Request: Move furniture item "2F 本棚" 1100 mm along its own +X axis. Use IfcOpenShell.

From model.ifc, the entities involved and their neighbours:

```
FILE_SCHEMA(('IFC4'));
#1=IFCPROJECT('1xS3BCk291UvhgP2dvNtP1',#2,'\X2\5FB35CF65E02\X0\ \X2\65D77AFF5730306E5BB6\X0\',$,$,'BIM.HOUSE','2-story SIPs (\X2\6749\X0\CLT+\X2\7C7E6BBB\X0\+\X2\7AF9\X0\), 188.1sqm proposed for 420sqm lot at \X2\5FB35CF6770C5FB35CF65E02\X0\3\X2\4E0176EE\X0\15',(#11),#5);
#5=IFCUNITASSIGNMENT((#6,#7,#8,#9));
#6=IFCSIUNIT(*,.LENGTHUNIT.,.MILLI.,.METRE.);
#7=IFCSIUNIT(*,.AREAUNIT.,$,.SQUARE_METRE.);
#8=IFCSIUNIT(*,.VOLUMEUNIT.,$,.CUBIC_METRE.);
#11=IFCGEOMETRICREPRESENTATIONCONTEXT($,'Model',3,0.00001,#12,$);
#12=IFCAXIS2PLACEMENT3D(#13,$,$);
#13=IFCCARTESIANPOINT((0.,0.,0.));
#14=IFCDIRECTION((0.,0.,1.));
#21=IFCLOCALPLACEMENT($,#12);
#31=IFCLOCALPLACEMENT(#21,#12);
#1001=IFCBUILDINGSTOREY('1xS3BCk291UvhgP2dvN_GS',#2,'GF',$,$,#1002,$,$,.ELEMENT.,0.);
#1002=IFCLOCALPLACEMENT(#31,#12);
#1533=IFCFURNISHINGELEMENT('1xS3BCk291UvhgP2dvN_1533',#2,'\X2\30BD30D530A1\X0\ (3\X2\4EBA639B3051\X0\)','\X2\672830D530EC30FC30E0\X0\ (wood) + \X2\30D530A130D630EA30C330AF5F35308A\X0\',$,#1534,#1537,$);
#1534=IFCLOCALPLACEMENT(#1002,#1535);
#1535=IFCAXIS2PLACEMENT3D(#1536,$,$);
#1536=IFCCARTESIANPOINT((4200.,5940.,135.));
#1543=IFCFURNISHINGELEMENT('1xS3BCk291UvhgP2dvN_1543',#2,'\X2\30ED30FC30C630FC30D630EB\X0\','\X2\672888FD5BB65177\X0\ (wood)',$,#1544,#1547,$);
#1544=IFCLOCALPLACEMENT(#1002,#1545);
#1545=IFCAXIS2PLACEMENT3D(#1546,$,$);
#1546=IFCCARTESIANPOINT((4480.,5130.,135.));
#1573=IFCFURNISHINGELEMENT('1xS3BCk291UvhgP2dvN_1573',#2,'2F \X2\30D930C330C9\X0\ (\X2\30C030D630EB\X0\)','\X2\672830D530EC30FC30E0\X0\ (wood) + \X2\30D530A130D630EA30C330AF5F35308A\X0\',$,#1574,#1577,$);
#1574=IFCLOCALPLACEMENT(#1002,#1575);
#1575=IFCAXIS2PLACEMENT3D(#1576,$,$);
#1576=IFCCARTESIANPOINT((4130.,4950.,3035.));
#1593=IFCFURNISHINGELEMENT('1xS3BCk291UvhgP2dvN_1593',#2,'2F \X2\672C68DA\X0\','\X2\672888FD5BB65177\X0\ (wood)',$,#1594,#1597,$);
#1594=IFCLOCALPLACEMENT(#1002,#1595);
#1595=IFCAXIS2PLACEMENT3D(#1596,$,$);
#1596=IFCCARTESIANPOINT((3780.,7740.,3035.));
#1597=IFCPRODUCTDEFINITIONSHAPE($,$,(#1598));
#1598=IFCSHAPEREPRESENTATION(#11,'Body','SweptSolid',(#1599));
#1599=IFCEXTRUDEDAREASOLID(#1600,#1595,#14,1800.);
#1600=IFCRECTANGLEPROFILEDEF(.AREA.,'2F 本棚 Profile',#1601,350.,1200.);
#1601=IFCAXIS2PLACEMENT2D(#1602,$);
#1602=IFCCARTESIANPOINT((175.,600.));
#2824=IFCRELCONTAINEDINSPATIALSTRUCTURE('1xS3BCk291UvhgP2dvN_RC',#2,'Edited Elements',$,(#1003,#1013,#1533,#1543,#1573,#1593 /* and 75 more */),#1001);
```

```python
import ifcopenshell
import ifcopenshell.api.geometry
import ifcopenshell.util.placement
import ifcopenshell.util.unit

model = ifcopenshell.open("model.ifc")
unit_scale = ifcopenshell.util.unit.calculate_unit_scale(model)

item = model.by_guid("1xS3BCk291UvhgP2dvN_1593")
matrix = ifcopenshell.util.placement.get_local_placement(item.ObjectPlacement)
matrix[:3, 3] += matrix[:3, 0] * 1.1 / unit_scale
ifcopenshell.api.geometry.edit_object_placement(model, product=item, matrix=matrix, is_si=False)

print(ifcopenshell.util.placement.get_local_placement(item.ObjectPlacement).round(3) + 0.0)

model.write("model_rev.ifc")
```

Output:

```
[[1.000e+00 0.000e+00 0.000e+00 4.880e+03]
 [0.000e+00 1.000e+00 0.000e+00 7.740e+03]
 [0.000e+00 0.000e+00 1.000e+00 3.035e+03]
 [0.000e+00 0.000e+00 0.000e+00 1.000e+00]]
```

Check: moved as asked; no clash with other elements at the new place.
